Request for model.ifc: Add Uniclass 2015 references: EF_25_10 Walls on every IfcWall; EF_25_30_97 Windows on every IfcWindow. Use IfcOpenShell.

First a look at what the model holds.

```python
import ifcopenshell

model = ifcopenshell.open("model.ifc")
print(model.schema)
print("classifications:", [c.Name for c in model.by_type("IfcClassification")])
for ifc_class in ("IfcDoor", "IfcRoof", "IfcStair", "IfcWall", "IfcWindow"):
    print(ifc_class, len(model.by_type(ifc_class)))
```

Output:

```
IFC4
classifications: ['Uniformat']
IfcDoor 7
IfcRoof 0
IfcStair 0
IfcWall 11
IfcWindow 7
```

```python
import ifcopenshell
import ifcopenshell.api.classification

model = ifcopenshell.open("model.ifc")

system = ifcopenshell.api.classification.add_classification(model, classification="Uniclass 2015")

codes = {
    "IfcWall": ("EF_25_10", "Walls"),
    "IfcWindow": ("EF_25_30_97", "Windows"),
}
for ifc_class, (code, name) in codes.items():
    products = model.by_type(ifc_class)
    ifcopenshell.api.classification.add_reference(
        model, products=products, classification=system, identification=code, name=name
    )
    print(code, len(products))

model.write("model_v2.ifc")
```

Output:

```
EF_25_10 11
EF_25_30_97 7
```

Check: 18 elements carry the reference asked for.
